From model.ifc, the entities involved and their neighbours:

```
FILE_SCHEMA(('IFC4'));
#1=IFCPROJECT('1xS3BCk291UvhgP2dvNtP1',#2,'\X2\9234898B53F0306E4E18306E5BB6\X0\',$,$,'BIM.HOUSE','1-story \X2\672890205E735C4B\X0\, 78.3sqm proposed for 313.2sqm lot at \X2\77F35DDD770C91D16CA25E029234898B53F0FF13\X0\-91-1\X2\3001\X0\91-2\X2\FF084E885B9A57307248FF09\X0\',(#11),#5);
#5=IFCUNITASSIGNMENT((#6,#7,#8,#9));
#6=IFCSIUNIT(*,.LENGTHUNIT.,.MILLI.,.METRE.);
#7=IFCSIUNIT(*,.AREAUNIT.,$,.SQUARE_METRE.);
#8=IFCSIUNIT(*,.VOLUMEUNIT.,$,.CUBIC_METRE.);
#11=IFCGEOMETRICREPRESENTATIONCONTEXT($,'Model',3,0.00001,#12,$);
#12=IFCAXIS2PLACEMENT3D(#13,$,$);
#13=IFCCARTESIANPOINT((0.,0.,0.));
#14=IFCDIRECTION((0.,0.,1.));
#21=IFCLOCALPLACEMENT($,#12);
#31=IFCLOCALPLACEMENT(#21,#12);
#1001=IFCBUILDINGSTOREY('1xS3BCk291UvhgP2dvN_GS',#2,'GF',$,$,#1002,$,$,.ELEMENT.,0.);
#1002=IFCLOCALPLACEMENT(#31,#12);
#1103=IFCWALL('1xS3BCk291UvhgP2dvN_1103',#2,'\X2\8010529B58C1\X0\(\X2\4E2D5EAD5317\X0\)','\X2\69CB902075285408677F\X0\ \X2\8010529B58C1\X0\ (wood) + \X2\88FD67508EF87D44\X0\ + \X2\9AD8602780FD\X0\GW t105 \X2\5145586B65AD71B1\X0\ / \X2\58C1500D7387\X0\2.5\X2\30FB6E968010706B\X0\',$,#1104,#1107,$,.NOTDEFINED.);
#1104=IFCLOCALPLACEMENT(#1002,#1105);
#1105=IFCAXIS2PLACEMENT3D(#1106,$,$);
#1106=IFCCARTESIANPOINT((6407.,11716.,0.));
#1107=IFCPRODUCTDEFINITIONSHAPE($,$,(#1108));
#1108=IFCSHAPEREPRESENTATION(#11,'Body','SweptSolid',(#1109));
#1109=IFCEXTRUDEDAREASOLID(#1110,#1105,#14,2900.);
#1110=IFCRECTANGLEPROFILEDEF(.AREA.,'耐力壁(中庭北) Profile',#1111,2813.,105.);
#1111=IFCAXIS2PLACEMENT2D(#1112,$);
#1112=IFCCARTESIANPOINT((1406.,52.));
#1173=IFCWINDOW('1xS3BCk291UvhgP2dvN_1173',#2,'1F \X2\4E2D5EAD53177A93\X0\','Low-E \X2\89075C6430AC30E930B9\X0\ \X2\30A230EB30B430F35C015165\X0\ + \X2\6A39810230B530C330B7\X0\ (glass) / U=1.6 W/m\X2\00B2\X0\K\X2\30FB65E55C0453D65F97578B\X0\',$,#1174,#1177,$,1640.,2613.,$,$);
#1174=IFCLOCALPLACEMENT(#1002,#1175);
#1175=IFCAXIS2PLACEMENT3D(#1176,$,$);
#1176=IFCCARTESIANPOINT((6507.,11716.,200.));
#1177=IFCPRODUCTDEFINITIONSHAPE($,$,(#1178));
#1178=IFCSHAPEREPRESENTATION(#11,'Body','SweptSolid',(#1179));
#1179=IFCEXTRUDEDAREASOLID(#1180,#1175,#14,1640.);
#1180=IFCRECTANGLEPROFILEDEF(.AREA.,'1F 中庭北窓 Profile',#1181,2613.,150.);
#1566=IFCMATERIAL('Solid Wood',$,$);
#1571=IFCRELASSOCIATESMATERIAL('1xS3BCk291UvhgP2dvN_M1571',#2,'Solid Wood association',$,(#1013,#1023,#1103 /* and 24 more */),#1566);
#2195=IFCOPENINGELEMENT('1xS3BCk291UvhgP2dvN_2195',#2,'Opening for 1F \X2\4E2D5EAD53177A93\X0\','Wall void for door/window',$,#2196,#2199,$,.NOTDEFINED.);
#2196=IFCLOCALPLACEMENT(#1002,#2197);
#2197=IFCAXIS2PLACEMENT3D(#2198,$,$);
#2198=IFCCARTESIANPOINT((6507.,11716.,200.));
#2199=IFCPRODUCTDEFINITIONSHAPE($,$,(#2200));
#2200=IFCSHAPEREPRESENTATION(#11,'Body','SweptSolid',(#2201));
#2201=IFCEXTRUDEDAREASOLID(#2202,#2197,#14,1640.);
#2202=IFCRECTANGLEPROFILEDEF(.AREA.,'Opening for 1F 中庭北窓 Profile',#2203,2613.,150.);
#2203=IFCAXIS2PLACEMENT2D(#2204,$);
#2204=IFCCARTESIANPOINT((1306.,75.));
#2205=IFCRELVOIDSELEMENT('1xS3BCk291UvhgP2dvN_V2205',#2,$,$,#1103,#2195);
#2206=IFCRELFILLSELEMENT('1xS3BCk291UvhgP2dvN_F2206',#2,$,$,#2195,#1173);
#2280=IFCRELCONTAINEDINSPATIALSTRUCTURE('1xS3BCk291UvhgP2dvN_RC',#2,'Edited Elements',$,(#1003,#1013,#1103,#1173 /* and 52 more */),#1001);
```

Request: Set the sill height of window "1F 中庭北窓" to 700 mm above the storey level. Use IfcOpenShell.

```python
import numpy as np
import ifcopenshell
import ifcopenshell.api.geometry
import ifcopenshell.geom
import ifcopenshell.util.element
import ifcopenshell.util.placement
import ifcopenshell.util.shape
import ifcopenshell.util.unit

model = ifcopenshell.open("model.ifc")
unit_scale = ifcopenshell.util.unit.calculate_unit_scale(model)

window = model.by_id(1173)
opening = window.FillsVoids[0].RelatingOpeningElement
storey = ifcopenshell.util.element.get_container(window, ifc_class="IfcBuildingStorey")
level = ifcopenshell.util.placement.get_local_placement(storey.ObjectPlacement)[2, 3]

# The opening's origin need not be at the sill, so measure its lowest point.
shape = ifcopenshell.geom.create_shape(ifcopenshell.geom.settings(), opening)
bottom = ifcopenshell.util.shape.get_shape_bottom_elevation(shape, shape.geometry) / unit_scale
dz = level + 700.0 - bottom

shift = np.array([0.0, 0.0, dz])
# The window is not placed relative to its opening, so move both.
for product in (opening, window):
    matrix = ifcopenshell.util.placement.get_local_placement(product.ObjectPlacement)
    matrix[:3, 3] += shift
    ifcopenshell.api.geometry.edit_object_placement(model, product=product, matrix=matrix, is_si=False)

print(f"moved by {dz * unit_scale:+.3f} m")

model.write("model-out.ifc")
```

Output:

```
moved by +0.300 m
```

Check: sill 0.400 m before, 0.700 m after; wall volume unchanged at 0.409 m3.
